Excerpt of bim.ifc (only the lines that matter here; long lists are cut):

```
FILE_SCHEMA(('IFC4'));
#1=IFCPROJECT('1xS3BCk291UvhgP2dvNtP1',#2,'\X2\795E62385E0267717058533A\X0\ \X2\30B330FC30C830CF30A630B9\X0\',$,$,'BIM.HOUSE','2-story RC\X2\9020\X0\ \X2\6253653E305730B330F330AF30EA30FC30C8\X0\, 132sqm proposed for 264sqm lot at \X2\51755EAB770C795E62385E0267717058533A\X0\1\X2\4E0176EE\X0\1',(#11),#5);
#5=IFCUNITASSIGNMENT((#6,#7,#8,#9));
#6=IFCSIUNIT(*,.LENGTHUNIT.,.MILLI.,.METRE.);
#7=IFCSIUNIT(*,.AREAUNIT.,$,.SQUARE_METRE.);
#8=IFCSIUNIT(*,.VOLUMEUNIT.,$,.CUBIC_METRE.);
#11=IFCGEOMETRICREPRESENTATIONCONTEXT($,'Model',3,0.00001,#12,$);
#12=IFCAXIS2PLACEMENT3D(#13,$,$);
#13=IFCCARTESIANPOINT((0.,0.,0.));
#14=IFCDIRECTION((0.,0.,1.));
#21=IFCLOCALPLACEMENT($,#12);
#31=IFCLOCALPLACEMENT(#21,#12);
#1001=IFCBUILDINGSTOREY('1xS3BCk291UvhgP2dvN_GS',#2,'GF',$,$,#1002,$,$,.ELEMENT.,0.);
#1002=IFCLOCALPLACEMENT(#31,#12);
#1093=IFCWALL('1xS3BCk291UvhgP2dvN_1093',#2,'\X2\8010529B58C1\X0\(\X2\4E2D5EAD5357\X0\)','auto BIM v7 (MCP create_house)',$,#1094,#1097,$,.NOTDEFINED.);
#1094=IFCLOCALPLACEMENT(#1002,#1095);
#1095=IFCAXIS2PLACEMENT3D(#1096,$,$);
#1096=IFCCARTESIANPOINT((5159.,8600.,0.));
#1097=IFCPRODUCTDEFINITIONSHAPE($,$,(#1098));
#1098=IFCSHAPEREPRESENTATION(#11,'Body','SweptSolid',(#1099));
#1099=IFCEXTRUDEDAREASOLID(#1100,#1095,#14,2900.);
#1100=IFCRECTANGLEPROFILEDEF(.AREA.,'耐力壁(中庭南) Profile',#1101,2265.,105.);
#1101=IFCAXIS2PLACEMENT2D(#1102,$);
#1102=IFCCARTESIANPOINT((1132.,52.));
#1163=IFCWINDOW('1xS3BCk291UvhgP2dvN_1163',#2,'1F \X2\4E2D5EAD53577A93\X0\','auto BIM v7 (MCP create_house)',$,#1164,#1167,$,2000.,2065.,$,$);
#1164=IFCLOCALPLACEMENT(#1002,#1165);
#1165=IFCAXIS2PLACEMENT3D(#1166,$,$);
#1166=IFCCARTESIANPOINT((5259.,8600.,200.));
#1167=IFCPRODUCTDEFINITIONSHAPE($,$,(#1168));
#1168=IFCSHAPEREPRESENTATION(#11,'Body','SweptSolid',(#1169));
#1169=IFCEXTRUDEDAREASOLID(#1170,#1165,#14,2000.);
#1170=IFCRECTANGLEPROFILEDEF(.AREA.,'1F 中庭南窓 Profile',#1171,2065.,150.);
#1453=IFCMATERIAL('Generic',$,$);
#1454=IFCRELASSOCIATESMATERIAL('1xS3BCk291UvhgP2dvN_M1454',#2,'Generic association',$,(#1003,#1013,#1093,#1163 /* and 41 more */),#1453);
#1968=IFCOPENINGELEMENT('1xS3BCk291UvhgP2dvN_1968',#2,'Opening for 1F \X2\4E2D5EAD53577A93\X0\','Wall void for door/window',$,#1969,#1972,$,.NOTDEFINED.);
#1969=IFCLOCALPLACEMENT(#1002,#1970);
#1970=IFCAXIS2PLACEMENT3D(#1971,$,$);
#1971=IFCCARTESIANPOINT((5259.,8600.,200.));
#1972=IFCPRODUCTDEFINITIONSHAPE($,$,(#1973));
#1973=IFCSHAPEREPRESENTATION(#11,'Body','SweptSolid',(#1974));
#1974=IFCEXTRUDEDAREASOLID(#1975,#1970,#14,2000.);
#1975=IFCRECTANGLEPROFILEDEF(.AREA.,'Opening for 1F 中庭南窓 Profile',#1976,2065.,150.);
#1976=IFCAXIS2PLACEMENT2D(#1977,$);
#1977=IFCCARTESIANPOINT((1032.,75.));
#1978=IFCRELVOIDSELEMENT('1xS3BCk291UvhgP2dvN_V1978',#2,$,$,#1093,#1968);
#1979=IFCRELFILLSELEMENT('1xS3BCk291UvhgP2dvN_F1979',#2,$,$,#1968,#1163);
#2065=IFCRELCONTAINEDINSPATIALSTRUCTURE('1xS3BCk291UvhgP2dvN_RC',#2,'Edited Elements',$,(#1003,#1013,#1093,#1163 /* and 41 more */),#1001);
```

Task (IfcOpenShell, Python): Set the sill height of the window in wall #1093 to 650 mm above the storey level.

```python
import numpy as np
import ifcopenshell
import ifcopenshell.api.geometry
import ifcopenshell.geom
import ifcopenshell.util.element
import ifcopenshell.util.placement
import ifcopenshell.util.shape
import ifcopenshell.util.unit

model = ifcopenshell.open("bim.ifc")
unit_scale = ifcopenshell.util.unit.calculate_unit_scale(model)

window = model.by_guid("1xS3BCk291UvhgP2dvN_1163")
opening = window.FillsVoids[0].RelatingOpeningElement
storey = ifcopenshell.util.element.get_container(window, ifc_class="IfcBuildingStorey")
level = ifcopenshell.util.placement.get_local_placement(storey.ObjectPlacement)[2, 3]

# The opening's origin need not be at the sill, so measure its lowest point.
shape = ifcopenshell.geom.create_shape(ifcopenshell.geom.settings(), opening)
bottom = ifcopenshell.util.shape.get_shape_bottom_elevation(shape, shape.geometry) / unit_scale
dz = level + 0.65 / unit_scale - bottom

shift = np.array([0.0, 0.0, dz])
# The window is not placed relative to its opening, so move both.
for product in (opening, window):
    matrix = ifcopenshell.util.placement.get_local_placement(product.ObjectPlacement)
    matrix[:3, 3] += shift
    ifcopenshell.api.geometry.edit_object_placement(model, product=product, matrix=matrix, is_si=False)

print(f"moved by {dz * unit_scale:+.3f} m")

model.write("bim_rev.ifc")
```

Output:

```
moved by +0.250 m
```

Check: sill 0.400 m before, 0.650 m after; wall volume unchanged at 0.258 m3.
